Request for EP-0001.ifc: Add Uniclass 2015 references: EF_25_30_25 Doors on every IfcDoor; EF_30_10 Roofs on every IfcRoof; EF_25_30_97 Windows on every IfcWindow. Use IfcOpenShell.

First a look at what the model holds.

```python
import ifcopenshell

model = ifcopenshell.open("EP-0001.ifc")
print(model.schema)
print("classifications:", [c.Name for c in model.by_type("IfcClassification")])
for ifc_class in ("IfcDoor", "IfcRoof", "IfcStair", "IfcWall", "IfcWindow"):
    print(ifc_class, len(model.by_type(ifc_class)))
```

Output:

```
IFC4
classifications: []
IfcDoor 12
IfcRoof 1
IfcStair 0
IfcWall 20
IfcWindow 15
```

```python
import ifcopenshell
import ifcopenshell.api.classification

model = ifcopenshell.open("EP-0001.ifc")

system = ifcopenshell.api.classification.add_classification(model, classification="Uniclass 2015")

codes = {
    "IfcDoor": ("EF_25_30_25", "Doors"),
    "IfcRoof": ("EF_30_10", "Roofs"),
    "IfcWindow": ("EF_25_30_97", "Windows"),
}
for ifc_class, (code, name) in codes.items():
    products = model.by_type(ifc_class)
    ifcopenshell.api.classification.add_reference(
        model, products=products, classification=system, identification=code, name=name
    )
    print(code, len(products))

model.write("EP-0001-out.ifc")
```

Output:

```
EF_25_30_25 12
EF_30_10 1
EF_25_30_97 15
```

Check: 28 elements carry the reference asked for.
